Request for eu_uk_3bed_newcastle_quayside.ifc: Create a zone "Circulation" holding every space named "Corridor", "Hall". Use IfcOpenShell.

First a look at what the model holds.

```python
import ifcopenshell

model = ifcopenshell.open("eu_uk_3bed_newcastle_quayside.ifc")
print(model.schema)
seen = {}
for space in model.by_type("IfcSpace"):
    seen[space.LongName] = seen.get(space.LongName, 0) + 1
for name, count in sorted(seen.items(), key=str):
    print(count, "x", name)
print("zones:", [z.Name for z in model.by_type("IfcZone")][:20])
```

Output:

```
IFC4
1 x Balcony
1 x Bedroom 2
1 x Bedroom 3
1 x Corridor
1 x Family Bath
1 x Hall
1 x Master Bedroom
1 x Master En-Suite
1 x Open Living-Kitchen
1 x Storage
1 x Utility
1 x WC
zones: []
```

```python
import ifcopenshell
import ifcopenshell.api.group
import ifcopenshell.api.root

model = ifcopenshell.open("eu_uk_3bed_newcastle_quayside.ifc")

names = {"Corridor", "Hall"}
spaces = [s for s in model.by_type("IfcSpace") if s.LongName in names]

zone = ifcopenshell.api.root.create_entity(model, ifc_class="IfcZone", name="Circulation")
ifcopenshell.api.group.assign_group(model, products=spaces, group=zone)
print(len(spaces), "spaces in", zone.Name)

model.write("eu_uk_3bed_newcastle_quayside_rev.ifc")
```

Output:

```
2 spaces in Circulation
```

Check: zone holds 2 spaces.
